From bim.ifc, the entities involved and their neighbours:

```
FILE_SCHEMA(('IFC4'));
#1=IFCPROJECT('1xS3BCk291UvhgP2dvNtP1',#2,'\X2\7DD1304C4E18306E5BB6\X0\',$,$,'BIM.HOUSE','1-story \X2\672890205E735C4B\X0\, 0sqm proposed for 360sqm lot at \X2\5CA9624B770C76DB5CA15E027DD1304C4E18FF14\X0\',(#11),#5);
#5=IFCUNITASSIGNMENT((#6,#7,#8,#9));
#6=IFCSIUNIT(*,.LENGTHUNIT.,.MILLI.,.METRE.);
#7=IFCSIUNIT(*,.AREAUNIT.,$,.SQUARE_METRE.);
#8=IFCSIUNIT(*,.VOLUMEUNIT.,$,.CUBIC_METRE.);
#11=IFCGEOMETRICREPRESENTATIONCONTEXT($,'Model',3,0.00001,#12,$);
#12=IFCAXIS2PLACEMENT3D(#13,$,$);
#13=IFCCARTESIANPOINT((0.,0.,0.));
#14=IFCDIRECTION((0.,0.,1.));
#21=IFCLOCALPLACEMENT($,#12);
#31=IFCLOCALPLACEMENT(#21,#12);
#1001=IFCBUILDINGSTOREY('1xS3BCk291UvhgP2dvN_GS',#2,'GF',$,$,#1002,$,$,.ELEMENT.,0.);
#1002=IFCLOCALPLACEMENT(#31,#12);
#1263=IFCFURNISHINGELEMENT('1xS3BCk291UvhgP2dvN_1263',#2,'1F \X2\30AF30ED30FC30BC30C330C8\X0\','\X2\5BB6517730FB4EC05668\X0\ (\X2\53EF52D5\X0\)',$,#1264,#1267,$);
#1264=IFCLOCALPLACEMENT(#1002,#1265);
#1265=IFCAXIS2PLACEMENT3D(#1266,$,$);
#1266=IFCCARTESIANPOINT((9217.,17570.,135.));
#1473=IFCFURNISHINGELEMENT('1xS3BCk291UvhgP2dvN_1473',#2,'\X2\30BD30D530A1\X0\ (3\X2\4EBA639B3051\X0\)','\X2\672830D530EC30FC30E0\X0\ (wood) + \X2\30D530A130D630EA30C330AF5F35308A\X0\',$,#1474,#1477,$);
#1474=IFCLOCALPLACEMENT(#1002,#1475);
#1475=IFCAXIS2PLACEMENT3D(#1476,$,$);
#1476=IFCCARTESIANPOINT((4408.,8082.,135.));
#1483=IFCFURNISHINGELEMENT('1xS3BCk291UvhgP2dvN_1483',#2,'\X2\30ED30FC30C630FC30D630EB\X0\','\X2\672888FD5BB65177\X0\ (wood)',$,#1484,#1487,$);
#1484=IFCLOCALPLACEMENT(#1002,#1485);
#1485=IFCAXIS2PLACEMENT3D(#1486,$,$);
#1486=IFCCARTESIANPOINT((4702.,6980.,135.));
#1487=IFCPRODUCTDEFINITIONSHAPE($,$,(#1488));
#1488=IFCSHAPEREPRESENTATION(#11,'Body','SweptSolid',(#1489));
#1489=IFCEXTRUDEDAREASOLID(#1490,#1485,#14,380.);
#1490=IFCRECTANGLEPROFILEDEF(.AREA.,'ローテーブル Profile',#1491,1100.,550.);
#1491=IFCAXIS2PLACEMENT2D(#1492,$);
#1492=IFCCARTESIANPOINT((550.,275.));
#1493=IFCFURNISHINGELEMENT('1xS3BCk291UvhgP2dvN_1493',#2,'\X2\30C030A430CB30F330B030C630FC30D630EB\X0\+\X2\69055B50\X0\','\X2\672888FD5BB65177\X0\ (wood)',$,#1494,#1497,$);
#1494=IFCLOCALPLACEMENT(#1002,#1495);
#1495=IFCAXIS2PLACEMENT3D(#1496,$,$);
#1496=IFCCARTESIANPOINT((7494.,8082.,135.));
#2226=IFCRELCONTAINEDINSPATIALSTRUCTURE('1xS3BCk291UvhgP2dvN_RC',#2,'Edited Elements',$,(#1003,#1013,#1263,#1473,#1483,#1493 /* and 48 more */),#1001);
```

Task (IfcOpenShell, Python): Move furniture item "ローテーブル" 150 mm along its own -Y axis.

```python
import ifcopenshell
import ifcopenshell.api.geometry
import ifcopenshell.util.placement
import ifcopenshell.util.unit

model = ifcopenshell.open("bim.ifc")
unit_scale = ifcopenshell.util.unit.calculate_unit_scale(model)

item = model.by_guid("1xS3BCk291UvhgP2dvN_1483")
matrix = ifcopenshell.util.placement.get_local_placement(item.ObjectPlacement)
matrix[:3, 3] -= matrix[:3, 1] * 0.15 / unit_scale
ifcopenshell.api.geometry.edit_object_placement(model, product=item, matrix=matrix, is_si=False)

print(ifcopenshell.util.placement.get_local_placement(item.ObjectPlacement).round(3) + 0.0)

model.write("bim_edited.ifc")
```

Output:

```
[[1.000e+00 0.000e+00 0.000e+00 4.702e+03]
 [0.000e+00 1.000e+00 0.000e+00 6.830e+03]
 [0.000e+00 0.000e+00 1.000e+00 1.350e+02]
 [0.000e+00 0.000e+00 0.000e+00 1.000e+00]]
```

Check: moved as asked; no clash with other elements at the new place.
